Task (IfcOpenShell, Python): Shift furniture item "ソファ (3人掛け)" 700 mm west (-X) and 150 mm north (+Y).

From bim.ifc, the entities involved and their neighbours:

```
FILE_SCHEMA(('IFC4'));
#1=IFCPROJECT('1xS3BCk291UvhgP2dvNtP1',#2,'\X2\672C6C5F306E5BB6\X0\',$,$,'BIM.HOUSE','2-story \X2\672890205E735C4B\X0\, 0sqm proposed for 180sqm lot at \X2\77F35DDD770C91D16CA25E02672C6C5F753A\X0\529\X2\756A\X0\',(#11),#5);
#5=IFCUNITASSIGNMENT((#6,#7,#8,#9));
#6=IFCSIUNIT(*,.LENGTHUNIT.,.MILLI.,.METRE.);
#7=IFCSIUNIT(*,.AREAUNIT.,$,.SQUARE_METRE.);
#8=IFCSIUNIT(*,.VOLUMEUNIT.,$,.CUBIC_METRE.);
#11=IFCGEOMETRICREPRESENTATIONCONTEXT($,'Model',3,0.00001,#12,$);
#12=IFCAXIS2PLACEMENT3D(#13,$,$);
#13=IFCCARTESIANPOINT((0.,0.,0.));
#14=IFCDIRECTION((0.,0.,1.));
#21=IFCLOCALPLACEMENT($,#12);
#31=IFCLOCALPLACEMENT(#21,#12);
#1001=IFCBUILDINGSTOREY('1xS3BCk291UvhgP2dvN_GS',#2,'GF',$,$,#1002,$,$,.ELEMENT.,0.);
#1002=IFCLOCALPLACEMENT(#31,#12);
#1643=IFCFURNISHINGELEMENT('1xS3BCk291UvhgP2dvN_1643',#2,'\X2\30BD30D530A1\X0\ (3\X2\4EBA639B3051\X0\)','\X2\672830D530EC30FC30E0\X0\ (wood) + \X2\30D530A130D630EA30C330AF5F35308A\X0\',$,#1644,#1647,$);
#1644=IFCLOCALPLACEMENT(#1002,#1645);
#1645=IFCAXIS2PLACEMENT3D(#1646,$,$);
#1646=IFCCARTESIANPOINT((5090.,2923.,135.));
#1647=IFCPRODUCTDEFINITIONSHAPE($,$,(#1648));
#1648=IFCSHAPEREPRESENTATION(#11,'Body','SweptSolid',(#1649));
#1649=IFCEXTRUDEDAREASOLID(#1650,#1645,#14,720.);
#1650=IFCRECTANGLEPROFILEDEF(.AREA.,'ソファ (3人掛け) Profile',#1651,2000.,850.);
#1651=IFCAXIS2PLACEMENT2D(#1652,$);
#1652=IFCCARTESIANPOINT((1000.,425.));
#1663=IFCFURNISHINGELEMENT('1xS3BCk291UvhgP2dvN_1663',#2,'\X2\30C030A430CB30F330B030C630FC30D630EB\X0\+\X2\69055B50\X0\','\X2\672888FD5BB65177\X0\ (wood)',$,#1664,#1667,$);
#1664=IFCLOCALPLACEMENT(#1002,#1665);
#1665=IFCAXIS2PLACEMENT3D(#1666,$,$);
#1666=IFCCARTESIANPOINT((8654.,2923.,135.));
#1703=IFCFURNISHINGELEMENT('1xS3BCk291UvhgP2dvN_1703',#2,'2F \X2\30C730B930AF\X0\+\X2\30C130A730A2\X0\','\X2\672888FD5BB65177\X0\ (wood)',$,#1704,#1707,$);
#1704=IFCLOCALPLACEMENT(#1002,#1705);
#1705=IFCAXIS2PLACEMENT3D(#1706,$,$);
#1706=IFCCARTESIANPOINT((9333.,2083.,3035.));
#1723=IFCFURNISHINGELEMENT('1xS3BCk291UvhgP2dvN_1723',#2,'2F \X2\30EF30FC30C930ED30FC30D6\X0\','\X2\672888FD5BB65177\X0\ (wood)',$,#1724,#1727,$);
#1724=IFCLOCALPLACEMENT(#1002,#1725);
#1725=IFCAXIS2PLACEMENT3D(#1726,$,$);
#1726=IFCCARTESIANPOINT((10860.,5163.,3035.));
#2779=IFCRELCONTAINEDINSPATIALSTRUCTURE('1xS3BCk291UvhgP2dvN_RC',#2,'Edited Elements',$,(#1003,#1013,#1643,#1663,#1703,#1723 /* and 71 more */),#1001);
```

```python
import ifcopenshell
import ifcopenshell.api.geometry
import ifcopenshell.util.placement
import ifcopenshell.util.unit

model = ifcopenshell.open("bim.ifc")
unit_scale = ifcopenshell.util.unit.calculate_unit_scale(model)

item = model.by_id(1643)
matrix = ifcopenshell.util.placement.get_local_placement(item.ObjectPlacement)
matrix[0, 3] -= 0.7 / unit_scale
matrix[1, 3] += 0.15 / unit_scale
ifcopenshell.api.geometry.edit_object_placement(model, product=item, matrix=matrix, is_si=False)

print(ifcopenshell.util.placement.get_local_placement(item.ObjectPlacement).round(3) + 0.0)

model.write("bim_rev.ifc")
```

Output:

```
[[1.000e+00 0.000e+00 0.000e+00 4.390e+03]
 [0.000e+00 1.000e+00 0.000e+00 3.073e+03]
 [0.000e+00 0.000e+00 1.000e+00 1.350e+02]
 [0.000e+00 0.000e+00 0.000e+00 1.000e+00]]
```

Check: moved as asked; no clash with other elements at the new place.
